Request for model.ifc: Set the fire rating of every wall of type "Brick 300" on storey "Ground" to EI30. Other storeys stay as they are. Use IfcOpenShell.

First a look at what the model holds.

```python
import ifcopenshell
import ifcopenshell.util.element

model = ifcopenshell.open("model.ifc")
print(model.schema)
storey = next(s for s in model.by_type("IfcBuildingStorey") if s.Name == "Ground")
walls = [e for e in ifcopenshell.util.element.get_decomposition(storey) if e.is_a("IfcWall")]
seen = {}
for e in walls:
    element_type = ifcopenshell.util.element.get_type(e)
    key = (element_type.Name if element_type != e and element_type else None, ifcopenshell.util.element.get_pset(e, "Pset_WallCommon", "FireRating"))
    seen[key] = seen.get(key, 0) + 1
for (name, value), count in sorted(seen.items(), key=str):
    print(count, "x", name, "|", value)
```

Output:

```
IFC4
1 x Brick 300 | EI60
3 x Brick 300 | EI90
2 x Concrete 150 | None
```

```python
import ifcopenshell
import ifcopenshell.api.pset
import ifcopenshell.util.element

model = ifcopenshell.open("model.ifc")

storey = next(s for s in model.by_type("IfcBuildingStorey") if s.Name == "Ground")
walls = [e for e in ifcopenshell.util.element.get_decomposition(storey) if e.is_a("IfcWall")]

count = 0
for e in walls:
    element_type = ifcopenshell.util.element.get_type(e)
    if element_type in (None, e) or element_type.Name != "Brick 300":
        continue
    # add_pset returns the element's existing set when there is one.
    pset = ifcopenshell.api.pset.add_pset(model, product=e, name="Pset_WallCommon")
    ifcopenshell.api.pset.edit_pset(model, pset=pset, properties={"FireRating": "EI30"})
    count += 1

print(count, "walls updated")

model.write("model_edited.ifc")
```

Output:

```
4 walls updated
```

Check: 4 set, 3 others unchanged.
